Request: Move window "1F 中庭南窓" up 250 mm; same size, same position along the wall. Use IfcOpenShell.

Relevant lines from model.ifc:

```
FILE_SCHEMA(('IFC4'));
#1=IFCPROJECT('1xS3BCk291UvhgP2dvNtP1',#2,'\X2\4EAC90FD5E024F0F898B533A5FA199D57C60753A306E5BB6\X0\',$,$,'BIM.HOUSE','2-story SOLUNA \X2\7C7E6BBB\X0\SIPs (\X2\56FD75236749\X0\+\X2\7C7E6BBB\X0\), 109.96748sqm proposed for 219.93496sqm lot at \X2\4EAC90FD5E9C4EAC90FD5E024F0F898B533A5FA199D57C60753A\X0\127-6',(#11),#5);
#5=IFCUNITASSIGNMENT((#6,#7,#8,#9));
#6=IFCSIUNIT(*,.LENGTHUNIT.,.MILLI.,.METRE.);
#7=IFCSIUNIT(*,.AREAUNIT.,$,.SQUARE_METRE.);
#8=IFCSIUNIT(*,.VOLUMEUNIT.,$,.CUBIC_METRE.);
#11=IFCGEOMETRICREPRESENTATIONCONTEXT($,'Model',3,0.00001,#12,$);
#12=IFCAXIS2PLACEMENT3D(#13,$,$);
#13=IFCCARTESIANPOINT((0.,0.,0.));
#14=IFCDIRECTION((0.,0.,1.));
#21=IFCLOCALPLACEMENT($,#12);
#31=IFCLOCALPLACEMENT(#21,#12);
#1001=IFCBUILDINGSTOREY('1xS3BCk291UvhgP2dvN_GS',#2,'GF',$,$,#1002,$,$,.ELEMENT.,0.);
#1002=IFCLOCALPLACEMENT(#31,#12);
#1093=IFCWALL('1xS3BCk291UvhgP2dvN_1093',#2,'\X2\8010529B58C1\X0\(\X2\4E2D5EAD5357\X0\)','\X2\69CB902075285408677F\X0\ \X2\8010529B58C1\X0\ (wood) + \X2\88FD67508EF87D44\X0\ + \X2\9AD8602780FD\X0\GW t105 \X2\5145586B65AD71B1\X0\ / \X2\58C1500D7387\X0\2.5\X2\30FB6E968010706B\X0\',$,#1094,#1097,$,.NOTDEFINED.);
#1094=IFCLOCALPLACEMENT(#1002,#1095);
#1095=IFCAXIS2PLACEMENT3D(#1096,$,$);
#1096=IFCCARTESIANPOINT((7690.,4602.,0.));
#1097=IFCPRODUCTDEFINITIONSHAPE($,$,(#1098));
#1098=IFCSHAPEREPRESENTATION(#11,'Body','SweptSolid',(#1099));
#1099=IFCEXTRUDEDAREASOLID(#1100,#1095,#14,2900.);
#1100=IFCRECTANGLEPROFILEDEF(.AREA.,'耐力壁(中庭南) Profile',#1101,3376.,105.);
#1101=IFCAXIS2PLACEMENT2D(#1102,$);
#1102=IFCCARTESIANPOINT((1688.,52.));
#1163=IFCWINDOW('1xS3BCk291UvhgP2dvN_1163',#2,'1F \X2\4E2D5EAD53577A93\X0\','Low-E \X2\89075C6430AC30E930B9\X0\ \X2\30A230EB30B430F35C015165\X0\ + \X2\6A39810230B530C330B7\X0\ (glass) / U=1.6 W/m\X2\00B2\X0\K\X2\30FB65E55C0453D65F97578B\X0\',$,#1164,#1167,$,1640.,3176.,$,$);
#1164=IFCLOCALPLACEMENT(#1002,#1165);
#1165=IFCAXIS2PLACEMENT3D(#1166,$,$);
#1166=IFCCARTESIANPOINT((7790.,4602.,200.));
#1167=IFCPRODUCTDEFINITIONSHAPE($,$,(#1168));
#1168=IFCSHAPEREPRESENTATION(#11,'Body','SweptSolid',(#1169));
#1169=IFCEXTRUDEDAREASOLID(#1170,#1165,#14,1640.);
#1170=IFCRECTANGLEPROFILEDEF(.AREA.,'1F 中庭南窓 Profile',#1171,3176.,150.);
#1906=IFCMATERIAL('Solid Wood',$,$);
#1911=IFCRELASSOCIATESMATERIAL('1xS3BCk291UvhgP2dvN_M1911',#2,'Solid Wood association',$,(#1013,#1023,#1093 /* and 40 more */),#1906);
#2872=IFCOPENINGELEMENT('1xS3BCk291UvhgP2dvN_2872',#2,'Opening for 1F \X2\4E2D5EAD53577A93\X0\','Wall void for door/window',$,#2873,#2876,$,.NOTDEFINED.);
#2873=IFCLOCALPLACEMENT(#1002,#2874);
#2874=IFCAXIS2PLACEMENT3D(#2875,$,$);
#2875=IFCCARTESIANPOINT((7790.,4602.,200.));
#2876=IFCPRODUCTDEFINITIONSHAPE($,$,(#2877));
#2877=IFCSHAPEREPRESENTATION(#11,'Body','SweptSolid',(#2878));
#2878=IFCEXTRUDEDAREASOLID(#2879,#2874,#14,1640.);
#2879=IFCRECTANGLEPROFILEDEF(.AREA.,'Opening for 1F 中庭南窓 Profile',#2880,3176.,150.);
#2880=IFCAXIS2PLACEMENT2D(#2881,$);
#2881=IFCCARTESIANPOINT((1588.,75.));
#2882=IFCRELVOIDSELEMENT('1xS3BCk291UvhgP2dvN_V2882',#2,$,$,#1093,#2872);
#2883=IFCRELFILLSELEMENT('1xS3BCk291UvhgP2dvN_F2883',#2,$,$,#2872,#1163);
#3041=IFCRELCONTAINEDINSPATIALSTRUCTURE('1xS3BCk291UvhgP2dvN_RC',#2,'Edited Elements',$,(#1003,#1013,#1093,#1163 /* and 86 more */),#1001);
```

```python
import numpy as np
import ifcopenshell
import ifcopenshell.api.geometry
import ifcopenshell.util.placement
import ifcopenshell.util.unit

model = ifcopenshell.open("model.ifc")
unit_scale = ifcopenshell.util.unit.calculate_unit_scale(model)

window = model.by_guid("1xS3BCk291UvhgP2dvN_1163")
opening = window.FillsVoids[0].RelatingOpeningElement
dz = 0.25 / unit_scale

shift = np.array([0.0, 0.0, dz])
# The window is not placed relative to its opening, so move both.
for product in (opening, window):
    matrix = ifcopenshell.util.placement.get_local_placement(product.ObjectPlacement)
    matrix[:3, 3] += shift
    ifcopenshell.api.geometry.edit_object_placement(model, product=product, matrix=matrix, is_si=False)

print(f"moved by {dz * unit_scale:+.3f} m")

model.write("model_updated.ifc")
```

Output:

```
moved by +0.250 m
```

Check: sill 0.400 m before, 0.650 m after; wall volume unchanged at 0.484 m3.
